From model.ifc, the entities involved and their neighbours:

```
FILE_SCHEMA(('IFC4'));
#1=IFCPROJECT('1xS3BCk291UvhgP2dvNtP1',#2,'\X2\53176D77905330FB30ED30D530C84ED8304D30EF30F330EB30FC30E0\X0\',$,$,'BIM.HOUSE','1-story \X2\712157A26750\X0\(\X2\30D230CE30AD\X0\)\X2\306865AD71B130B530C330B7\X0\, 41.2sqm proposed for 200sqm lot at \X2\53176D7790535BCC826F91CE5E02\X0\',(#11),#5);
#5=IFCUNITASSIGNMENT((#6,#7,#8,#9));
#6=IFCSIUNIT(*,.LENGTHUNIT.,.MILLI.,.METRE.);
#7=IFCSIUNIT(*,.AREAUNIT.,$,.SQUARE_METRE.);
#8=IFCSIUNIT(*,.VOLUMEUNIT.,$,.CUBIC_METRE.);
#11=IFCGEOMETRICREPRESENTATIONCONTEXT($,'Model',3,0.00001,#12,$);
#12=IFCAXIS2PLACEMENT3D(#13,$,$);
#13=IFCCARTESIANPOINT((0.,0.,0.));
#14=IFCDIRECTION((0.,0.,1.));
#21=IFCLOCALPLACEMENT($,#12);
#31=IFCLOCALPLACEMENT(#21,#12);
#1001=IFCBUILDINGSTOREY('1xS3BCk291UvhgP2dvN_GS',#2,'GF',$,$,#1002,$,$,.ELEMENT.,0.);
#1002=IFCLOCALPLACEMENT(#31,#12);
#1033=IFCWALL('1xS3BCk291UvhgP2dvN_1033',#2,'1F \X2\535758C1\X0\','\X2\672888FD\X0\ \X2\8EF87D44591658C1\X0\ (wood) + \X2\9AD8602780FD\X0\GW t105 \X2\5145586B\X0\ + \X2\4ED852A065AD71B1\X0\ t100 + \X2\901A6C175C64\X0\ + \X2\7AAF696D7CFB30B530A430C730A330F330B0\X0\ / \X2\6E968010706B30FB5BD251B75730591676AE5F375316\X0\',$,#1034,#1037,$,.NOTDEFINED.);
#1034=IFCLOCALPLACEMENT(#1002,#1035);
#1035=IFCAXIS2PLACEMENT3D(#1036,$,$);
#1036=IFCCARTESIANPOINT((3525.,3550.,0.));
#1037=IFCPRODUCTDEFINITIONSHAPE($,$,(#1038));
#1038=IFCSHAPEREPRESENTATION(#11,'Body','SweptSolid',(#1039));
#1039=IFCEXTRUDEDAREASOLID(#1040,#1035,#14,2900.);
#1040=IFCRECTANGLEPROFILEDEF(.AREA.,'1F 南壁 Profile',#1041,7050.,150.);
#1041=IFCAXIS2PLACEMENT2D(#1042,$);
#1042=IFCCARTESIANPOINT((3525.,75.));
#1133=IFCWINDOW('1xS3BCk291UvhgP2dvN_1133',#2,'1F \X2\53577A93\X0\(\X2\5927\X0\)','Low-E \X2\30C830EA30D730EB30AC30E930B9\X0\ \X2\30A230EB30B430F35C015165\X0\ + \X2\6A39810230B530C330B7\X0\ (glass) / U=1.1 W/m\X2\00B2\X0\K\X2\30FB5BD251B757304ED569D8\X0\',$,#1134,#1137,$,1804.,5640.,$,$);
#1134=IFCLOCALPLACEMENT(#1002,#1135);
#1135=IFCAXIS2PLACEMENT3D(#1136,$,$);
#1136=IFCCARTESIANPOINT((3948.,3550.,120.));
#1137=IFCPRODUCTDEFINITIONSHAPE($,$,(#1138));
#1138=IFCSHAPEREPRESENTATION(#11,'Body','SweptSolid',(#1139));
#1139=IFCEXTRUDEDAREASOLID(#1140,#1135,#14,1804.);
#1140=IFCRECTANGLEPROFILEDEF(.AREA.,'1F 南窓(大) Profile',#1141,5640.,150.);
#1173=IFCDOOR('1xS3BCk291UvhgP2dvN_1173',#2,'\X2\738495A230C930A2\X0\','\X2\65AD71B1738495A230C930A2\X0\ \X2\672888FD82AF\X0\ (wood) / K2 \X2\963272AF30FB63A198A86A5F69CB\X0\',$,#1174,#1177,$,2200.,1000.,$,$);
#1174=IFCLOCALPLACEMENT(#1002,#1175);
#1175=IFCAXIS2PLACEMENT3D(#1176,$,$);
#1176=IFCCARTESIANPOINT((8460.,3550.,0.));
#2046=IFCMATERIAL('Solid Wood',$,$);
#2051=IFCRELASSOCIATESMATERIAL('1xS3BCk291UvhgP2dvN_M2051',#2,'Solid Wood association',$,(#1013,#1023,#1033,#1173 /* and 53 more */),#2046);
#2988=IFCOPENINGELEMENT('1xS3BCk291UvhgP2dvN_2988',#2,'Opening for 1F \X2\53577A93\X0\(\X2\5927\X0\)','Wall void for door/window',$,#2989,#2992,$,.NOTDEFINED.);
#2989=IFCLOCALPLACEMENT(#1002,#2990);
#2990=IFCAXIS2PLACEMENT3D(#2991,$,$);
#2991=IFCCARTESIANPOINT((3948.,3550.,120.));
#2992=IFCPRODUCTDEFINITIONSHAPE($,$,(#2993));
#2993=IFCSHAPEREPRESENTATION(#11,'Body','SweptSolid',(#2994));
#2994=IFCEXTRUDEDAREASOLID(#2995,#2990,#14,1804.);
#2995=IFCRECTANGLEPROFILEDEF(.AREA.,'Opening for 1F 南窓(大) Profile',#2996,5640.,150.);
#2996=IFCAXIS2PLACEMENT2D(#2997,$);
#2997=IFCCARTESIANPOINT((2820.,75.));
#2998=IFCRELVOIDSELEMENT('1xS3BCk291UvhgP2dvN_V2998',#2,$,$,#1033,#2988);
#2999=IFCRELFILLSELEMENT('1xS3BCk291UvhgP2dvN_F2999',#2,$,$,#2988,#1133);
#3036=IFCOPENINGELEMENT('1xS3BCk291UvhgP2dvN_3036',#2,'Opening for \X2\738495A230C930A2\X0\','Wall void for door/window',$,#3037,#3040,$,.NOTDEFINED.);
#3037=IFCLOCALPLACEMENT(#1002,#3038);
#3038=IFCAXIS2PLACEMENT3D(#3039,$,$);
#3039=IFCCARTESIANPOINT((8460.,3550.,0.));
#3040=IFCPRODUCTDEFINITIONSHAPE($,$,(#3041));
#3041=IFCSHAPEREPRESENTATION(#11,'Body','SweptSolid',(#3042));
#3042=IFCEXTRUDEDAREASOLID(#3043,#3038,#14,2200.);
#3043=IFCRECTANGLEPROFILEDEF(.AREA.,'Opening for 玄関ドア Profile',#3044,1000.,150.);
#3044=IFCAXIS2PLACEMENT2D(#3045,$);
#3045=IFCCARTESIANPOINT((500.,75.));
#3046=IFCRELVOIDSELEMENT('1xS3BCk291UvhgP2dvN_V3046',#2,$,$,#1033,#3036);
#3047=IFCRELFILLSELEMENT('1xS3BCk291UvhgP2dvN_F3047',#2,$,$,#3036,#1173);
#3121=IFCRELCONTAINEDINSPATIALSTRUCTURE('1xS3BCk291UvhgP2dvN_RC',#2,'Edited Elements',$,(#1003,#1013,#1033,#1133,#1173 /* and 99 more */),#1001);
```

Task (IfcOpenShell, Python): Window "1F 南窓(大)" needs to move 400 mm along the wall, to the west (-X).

```python
import ifcopenshell
import ifcopenshell.api.geometry
import ifcopenshell.util.placement
import ifcopenshell.util.unit

model = ifcopenshell.open("model.ifc")
unit_scale = ifcopenshell.util.unit.calculate_unit_scale(model)

window = model.by_guid("1xS3BCk291UvhgP2dvN_1133")
opening = window.FillsVoids[0].RelatingOpeningElement
wall = opening.VoidsElements[0].RelatingBuildingElement

wall_matrix = ifcopenshell.util.placement.get_local_placement(wall.ObjectPlacement)
shift = wall_matrix[:3, 0] * -0.4 / unit_scale
before = ifcopenshell.util.placement.get_local_placement(window.ObjectPlacement)[:3, 3].copy()

# The window is not placed relative to its opening, so move both.
for product in (opening, window):
    matrix = ifcopenshell.util.placement.get_local_placement(product.ObjectPlacement)
    matrix[:3, 3] += shift
    ifcopenshell.api.geometry.edit_object_placement(model, product=product, matrix=matrix, is_si=False)

after = ifcopenshell.util.placement.get_local_placement(window.ObjectPlacement)[:3, 3]
print("window moved by", (after - before).round(3) + 0.0)

model.write("model_rev.ifc")
```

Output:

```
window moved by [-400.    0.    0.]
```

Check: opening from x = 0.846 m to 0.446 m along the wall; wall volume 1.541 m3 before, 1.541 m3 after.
